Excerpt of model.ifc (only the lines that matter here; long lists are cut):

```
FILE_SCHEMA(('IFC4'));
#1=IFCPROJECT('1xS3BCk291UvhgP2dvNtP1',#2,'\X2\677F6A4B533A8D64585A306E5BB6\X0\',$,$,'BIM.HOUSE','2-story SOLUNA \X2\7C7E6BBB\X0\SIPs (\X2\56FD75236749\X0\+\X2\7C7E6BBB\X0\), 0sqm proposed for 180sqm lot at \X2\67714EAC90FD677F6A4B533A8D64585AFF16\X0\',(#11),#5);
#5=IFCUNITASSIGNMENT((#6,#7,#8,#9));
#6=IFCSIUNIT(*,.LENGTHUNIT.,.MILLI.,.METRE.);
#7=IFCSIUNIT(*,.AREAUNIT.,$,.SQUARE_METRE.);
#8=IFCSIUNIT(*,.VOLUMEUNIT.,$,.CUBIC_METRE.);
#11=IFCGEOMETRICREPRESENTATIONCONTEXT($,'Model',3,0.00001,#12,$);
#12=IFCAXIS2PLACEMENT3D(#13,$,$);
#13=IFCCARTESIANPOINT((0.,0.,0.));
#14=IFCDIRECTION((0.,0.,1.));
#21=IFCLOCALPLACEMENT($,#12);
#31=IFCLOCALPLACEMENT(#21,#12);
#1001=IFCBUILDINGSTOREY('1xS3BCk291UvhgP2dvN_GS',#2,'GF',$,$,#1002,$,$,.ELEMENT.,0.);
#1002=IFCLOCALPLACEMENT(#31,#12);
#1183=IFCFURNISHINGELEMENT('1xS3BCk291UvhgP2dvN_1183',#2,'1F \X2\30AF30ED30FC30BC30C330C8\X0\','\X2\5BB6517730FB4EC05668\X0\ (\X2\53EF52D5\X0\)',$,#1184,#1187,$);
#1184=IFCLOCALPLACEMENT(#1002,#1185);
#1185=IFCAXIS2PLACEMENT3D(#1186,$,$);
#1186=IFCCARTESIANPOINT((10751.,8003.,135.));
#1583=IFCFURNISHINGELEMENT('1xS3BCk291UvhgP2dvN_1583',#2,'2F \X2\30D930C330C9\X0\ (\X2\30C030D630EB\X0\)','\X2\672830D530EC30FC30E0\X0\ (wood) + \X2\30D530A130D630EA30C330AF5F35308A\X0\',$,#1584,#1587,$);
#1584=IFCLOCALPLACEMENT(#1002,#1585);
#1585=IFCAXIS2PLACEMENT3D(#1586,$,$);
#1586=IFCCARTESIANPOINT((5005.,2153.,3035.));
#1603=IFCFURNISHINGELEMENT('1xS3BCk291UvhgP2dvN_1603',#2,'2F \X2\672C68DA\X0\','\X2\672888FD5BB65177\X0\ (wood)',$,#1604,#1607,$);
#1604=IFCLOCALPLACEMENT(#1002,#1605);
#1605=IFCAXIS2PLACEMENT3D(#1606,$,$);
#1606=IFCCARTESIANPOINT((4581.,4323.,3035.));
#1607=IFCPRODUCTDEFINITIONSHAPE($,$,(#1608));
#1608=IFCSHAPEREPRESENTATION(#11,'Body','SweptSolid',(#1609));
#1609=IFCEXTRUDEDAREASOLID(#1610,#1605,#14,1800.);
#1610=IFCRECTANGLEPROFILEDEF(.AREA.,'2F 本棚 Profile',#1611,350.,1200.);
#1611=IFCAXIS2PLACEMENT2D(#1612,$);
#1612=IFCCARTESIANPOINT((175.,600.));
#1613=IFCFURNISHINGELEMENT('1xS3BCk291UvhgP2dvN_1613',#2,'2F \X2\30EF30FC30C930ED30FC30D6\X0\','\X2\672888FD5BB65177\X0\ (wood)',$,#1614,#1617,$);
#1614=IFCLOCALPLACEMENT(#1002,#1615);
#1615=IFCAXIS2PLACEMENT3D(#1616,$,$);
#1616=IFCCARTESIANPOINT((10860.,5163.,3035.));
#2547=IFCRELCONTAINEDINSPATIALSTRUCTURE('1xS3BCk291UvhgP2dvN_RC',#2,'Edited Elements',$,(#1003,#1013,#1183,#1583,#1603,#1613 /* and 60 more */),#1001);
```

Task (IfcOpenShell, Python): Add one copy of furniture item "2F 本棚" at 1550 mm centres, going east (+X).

```python
import numpy as np
import ifcopenshell
import ifcopenshell.api.geometry
import ifcopenshell.api.root
import ifcopenshell.util.element
import ifcopenshell.util.placement

model = ifcopenshell.open("model.ifc")


def reuse_history(source, copy):
    """copy_class also copies each property set's owner history, people and application; keep the originals."""
    for rel in copy.IsDefinedBy:
        if rel.is_a("IfcRelDefinesByProperties") and (history := rel.RelatingPropertyDefinition.OwnerHistory):
            rel.RelatingPropertyDefinition.OwnerHistory = source.OwnerHistory
            ifcopenshell.util.element.remove_deep2(model, history)


source = model.by_guid("1xS3BCk291UvhgP2dvN_1603")
base = ifcopenshell.util.placement.get_local_placement(source.ObjectPlacement)
step = np.array([1.0, 0.0, 0.0]) * 1550.0

for i in range(1, 2):
    copy = ifcopenshell.api.root.copy_class(model, product=source)
    copy.Representation = ifcopenshell.util.element.copy_deep(
        model, source.Representation, exclude=["IfcGeometricRepresentationContext", "IfcRepresentationMap"]
    )
    reuse_history(source, copy)
    matrix = base.copy()
    matrix[:3, 3] += i * step
    print("added at", matrix[:3, 3].round(3) + 0.0)
    ifcopenshell.api.geometry.edit_object_placement(model, product=copy, matrix=matrix, is_si=False)

model.write("model_v2.ifc")
```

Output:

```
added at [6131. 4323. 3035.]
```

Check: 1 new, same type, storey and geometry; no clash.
